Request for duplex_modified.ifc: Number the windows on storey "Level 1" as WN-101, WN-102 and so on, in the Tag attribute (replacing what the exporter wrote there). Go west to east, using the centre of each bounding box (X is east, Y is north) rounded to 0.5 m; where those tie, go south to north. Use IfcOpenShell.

First a look at what the model holds.

```python
import ifcopenshell
import ifcopenshell.util.element
import ifcopenshell.util.placement

model = ifcopenshell.open("duplex_modified.ifc")
print(model.schema)
storey = next(s for s in model.by_type("IfcBuildingStorey") if s.Name == "Level 1")
windows = [e for e in ifcopenshell.util.element.get_decomposition(storey) if e.is_a("IfcWindow")]
for e in sorted(windows, key=lambda e: e.id()):
    origin = ifcopenshell.util.placement.get_local_placement(e.ObjectPlacement)[:3, 3]
    print(e.id(), e.Tag, e.Name, origin.round(2) + 0.0, sep=" | ")
```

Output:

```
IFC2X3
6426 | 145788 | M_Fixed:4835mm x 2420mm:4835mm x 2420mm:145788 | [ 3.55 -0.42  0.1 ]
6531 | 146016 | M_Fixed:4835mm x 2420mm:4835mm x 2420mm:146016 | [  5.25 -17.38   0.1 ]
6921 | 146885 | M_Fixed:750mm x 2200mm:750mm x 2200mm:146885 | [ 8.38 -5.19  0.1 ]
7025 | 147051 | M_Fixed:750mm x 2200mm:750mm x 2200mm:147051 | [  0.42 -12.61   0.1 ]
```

```python
import ifcopenshell
import ifcopenshell.geom
import ifcopenshell.util.element
import ifcopenshell.util.shape

model = ifcopenshell.open("duplex_modified.ifc")
settings = ifcopenshell.geom.settings()
settings.set("use-world-coords", True)


def centre(element):
    shape = ifcopenshell.geom.create_shape(settings, element)
    return ifcopenshell.util.shape.get_bbox_centroid(shape.geometry)


storey = next(s for s in model.by_type("IfcBuildingStorey") if s.Name == "Level 1")
windows = [e for e in ifcopenshell.util.element.get_decomposition(storey) if e.is_a("IfcWindow")]

# Insertion points can sit at a corner or the storey origin, so sort by the geometry (in metres).
centres = {e: centre(e) for e in windows}
windows.sort(key=lambda e: (round(centres[e][0] / 0.5), centres[e][1]))

for i, e in enumerate(windows, start=1):
    number = f"WN-1{i:02d}"
    e.Tag = number
    print(e.id(), number)

model.write("duplex_modified_edited.ifc")
```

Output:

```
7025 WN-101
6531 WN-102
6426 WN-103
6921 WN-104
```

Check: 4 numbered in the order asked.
